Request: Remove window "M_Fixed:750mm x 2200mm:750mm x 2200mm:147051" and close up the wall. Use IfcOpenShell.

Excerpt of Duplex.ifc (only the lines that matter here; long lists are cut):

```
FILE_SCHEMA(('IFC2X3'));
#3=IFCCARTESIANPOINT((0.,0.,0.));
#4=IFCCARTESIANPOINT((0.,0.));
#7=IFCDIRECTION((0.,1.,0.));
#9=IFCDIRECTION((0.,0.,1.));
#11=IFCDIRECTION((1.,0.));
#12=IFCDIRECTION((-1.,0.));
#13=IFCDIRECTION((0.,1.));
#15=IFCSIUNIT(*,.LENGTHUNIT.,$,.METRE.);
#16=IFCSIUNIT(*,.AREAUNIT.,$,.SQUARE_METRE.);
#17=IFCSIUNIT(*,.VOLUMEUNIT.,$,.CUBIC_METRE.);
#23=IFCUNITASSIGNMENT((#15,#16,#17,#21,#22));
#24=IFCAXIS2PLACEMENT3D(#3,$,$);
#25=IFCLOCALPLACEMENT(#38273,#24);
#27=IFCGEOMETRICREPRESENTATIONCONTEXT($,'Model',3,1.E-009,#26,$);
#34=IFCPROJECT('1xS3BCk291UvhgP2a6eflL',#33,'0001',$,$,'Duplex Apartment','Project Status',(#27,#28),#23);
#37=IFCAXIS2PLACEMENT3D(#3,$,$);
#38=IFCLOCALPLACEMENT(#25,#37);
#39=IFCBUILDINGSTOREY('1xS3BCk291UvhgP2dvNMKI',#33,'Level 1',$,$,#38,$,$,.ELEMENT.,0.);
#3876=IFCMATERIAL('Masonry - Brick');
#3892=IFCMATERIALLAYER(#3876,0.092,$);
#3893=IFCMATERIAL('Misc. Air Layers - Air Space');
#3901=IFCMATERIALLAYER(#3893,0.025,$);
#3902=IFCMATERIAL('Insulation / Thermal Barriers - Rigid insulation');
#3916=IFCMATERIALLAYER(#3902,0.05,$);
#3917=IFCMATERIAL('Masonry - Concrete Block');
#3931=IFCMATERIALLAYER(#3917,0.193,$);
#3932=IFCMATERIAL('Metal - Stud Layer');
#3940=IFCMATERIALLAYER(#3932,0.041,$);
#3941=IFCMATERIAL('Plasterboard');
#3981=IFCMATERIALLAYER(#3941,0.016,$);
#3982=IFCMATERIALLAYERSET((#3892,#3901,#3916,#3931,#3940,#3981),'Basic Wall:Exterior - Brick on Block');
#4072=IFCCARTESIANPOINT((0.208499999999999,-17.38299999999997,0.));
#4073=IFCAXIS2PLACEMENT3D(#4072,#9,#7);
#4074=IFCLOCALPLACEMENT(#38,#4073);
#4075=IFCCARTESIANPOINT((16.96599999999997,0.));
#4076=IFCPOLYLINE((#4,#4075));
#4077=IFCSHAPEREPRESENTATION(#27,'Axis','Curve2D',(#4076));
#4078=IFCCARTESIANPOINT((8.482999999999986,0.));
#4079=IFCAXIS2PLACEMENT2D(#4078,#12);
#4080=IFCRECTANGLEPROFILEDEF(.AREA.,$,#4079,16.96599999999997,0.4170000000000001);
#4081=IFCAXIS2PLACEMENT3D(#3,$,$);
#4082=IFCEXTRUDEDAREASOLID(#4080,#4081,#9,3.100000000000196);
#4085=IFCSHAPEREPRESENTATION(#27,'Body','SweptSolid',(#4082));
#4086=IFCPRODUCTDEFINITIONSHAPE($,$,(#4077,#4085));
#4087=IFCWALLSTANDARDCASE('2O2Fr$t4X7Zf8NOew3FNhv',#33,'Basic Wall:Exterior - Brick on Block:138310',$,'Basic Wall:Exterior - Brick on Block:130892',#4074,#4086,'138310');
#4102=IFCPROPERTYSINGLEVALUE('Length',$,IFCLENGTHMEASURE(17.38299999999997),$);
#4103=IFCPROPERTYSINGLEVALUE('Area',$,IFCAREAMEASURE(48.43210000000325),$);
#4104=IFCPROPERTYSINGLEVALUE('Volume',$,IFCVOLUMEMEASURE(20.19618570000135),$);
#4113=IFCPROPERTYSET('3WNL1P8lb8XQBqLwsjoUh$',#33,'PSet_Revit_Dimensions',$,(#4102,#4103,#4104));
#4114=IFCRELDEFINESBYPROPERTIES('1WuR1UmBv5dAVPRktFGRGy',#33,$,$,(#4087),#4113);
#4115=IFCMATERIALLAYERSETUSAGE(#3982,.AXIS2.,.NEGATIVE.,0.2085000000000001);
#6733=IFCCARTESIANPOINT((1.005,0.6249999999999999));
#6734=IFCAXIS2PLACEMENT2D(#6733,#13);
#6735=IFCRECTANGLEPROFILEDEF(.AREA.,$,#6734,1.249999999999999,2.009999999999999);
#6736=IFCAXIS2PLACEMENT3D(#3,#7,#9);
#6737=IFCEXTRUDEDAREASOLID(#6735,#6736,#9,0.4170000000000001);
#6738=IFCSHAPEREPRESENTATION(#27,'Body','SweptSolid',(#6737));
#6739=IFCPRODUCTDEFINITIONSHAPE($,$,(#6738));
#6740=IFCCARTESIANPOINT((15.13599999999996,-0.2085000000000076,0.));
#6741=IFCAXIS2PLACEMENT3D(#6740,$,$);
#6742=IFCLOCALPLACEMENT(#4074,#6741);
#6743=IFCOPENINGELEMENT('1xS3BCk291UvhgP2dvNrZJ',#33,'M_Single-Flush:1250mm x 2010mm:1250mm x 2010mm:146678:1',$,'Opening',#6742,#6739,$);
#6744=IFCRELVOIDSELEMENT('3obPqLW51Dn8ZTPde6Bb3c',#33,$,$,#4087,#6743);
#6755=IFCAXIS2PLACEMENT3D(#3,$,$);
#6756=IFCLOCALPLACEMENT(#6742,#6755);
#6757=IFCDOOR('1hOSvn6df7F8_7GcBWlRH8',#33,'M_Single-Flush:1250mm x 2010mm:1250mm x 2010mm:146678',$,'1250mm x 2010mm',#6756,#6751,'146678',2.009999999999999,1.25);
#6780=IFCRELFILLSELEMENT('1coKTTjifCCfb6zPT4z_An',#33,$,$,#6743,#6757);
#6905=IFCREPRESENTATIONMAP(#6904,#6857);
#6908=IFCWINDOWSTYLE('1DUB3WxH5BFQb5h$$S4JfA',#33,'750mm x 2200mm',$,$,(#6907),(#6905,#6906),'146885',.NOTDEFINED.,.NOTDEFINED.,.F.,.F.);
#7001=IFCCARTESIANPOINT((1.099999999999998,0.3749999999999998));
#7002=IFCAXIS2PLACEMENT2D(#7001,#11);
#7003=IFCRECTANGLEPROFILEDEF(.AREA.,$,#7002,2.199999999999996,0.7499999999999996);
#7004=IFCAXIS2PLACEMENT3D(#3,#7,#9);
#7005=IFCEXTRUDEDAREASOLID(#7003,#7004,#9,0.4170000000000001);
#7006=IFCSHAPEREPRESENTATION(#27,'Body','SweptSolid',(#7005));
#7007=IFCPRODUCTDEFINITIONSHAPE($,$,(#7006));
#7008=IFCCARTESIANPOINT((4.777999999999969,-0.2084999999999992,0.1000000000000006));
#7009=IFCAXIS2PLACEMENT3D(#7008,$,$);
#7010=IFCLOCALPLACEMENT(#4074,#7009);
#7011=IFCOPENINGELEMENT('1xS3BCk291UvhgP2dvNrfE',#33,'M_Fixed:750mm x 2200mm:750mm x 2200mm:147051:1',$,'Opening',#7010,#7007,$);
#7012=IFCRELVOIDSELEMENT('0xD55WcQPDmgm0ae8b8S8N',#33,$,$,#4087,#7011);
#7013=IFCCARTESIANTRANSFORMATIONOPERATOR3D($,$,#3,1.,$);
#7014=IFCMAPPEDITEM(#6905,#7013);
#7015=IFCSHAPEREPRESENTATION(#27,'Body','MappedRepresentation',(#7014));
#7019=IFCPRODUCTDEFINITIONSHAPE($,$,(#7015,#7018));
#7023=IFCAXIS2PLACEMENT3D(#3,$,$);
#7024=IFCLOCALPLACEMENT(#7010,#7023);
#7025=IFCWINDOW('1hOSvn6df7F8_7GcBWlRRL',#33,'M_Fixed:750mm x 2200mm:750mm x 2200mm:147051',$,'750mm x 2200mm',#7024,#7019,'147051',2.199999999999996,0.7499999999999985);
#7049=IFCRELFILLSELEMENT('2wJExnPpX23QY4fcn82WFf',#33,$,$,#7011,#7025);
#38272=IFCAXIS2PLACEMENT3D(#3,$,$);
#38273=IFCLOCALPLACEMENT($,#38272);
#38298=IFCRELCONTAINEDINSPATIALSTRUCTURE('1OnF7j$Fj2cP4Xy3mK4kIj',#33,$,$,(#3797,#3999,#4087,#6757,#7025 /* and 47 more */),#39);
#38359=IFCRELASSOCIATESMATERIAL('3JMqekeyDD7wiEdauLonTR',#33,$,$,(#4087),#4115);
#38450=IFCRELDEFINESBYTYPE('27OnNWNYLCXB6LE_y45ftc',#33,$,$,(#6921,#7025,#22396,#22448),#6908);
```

```python
import ifcopenshell
import ifcopenshell.api.feature
import ifcopenshell.api.pset
import ifcopenshell.api.root
import ifcopenshell.geom
import ifcopenshell.util.element
import ifcopenshell.util.shape
import ifcopenshell.util.unit

model = ifcopenshell.open("Duplex.ifc")
area_scale = ifcopenshell.util.unit.calculate_unit_scale(model, "AREAUNIT")
volume_scale = ifcopenshell.util.unit.calculate_unit_scale(model, "VOLUMEUNIT")
settings = ifcopenshell.geom.settings()


def volume(element):
    """Net volume in cubic metres, openings subtracted."""
    shape = ifcopenshell.geom.create_shape(settings, element)
    return ifcopenshell.util.shape.get_volume(shape.geometry)


window = model.by_guid("1hOSvn6df7F8_7GcBWlRRL")
opening = window.FillsVoids[0].RelatingOpeningElement
wall = opening.VoidsElements[0].RelatingBuildingElement
before = volume(wall)

ifcopenshell.api.root.remove_product(model, product=window)
ifcopenshell.api.feature.remove_feature(model, feature=opening)

after = volume(wall)
thickness = 0.417  # wall thickness in metres

# Update the wall's stored quantities.
pset = model.by_id(ifcopenshell.util.element.get_pset(wall, "PSet_Revit_Dimensions", should_inherit=False)["id"])
ifcopenshell.api.pset.edit_pset(model, pset=pset, properties={
    "Area": model.create_entity("IfcAreaMeasure", after / thickness / area_scale),
    "Volume": model.create_entity("IfcVolumeMeasure", after / volume_scale),
})

print(f"wall volume {before:.3f} -> {after:.3f} m3")

model.write("Duplex_v2.ifc")
```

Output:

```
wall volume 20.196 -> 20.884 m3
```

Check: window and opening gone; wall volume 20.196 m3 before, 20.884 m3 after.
